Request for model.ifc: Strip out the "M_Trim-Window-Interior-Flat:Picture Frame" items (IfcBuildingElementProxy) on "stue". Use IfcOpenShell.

First a look at what the model holds.

```python
import ifcopenshell
import ifcopenshell.util.element

model = ifcopenshell.open("model.ifc")
print(model.schema)
storey = next(s for s in model.by_type("IfcBuildingStorey") if s.Name == "stue")
proxies = [e for e in ifcopenshell.util.element.get_decomposition(storey) if e.is_a("IfcBuildingElementProxy")]
seen = {}
for e in proxies:
    element_type = ifcopenshell.util.element.get_type(e)
    name = element_type.Name if element_type not in (None, e) else None
    seen[name] = seen.get(name, 0) + 1
for name, count in sorted(seen.items(), key=str):
    print(count, "x", name)
```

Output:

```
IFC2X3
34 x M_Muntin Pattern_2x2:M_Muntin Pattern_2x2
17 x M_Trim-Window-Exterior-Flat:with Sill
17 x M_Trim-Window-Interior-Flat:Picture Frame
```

```python
import ifcopenshell
import ifcopenshell.api.root
import ifcopenshell.util.element

model = ifcopenshell.open("model.ifc")

storey = next(s for s in model.by_type("IfcBuildingStorey") if s.Name == "stue")
proxies = [e for e in ifcopenshell.util.element.get_decomposition(storey) if e.is_a("IfcBuildingElementProxy")]
targets = [e for e in proxies if (t := ifcopenshell.util.element.get_type(e)) not in (None, e) and t.Name == "M_Trim-Window-Interior-Flat:Picture Frame"]

for e in targets:
    ifcopenshell.api.root.remove_product(model, product=e)
print(len(targets), "removed")

model.write("model_updated.ifc")
```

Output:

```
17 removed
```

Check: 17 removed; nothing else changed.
